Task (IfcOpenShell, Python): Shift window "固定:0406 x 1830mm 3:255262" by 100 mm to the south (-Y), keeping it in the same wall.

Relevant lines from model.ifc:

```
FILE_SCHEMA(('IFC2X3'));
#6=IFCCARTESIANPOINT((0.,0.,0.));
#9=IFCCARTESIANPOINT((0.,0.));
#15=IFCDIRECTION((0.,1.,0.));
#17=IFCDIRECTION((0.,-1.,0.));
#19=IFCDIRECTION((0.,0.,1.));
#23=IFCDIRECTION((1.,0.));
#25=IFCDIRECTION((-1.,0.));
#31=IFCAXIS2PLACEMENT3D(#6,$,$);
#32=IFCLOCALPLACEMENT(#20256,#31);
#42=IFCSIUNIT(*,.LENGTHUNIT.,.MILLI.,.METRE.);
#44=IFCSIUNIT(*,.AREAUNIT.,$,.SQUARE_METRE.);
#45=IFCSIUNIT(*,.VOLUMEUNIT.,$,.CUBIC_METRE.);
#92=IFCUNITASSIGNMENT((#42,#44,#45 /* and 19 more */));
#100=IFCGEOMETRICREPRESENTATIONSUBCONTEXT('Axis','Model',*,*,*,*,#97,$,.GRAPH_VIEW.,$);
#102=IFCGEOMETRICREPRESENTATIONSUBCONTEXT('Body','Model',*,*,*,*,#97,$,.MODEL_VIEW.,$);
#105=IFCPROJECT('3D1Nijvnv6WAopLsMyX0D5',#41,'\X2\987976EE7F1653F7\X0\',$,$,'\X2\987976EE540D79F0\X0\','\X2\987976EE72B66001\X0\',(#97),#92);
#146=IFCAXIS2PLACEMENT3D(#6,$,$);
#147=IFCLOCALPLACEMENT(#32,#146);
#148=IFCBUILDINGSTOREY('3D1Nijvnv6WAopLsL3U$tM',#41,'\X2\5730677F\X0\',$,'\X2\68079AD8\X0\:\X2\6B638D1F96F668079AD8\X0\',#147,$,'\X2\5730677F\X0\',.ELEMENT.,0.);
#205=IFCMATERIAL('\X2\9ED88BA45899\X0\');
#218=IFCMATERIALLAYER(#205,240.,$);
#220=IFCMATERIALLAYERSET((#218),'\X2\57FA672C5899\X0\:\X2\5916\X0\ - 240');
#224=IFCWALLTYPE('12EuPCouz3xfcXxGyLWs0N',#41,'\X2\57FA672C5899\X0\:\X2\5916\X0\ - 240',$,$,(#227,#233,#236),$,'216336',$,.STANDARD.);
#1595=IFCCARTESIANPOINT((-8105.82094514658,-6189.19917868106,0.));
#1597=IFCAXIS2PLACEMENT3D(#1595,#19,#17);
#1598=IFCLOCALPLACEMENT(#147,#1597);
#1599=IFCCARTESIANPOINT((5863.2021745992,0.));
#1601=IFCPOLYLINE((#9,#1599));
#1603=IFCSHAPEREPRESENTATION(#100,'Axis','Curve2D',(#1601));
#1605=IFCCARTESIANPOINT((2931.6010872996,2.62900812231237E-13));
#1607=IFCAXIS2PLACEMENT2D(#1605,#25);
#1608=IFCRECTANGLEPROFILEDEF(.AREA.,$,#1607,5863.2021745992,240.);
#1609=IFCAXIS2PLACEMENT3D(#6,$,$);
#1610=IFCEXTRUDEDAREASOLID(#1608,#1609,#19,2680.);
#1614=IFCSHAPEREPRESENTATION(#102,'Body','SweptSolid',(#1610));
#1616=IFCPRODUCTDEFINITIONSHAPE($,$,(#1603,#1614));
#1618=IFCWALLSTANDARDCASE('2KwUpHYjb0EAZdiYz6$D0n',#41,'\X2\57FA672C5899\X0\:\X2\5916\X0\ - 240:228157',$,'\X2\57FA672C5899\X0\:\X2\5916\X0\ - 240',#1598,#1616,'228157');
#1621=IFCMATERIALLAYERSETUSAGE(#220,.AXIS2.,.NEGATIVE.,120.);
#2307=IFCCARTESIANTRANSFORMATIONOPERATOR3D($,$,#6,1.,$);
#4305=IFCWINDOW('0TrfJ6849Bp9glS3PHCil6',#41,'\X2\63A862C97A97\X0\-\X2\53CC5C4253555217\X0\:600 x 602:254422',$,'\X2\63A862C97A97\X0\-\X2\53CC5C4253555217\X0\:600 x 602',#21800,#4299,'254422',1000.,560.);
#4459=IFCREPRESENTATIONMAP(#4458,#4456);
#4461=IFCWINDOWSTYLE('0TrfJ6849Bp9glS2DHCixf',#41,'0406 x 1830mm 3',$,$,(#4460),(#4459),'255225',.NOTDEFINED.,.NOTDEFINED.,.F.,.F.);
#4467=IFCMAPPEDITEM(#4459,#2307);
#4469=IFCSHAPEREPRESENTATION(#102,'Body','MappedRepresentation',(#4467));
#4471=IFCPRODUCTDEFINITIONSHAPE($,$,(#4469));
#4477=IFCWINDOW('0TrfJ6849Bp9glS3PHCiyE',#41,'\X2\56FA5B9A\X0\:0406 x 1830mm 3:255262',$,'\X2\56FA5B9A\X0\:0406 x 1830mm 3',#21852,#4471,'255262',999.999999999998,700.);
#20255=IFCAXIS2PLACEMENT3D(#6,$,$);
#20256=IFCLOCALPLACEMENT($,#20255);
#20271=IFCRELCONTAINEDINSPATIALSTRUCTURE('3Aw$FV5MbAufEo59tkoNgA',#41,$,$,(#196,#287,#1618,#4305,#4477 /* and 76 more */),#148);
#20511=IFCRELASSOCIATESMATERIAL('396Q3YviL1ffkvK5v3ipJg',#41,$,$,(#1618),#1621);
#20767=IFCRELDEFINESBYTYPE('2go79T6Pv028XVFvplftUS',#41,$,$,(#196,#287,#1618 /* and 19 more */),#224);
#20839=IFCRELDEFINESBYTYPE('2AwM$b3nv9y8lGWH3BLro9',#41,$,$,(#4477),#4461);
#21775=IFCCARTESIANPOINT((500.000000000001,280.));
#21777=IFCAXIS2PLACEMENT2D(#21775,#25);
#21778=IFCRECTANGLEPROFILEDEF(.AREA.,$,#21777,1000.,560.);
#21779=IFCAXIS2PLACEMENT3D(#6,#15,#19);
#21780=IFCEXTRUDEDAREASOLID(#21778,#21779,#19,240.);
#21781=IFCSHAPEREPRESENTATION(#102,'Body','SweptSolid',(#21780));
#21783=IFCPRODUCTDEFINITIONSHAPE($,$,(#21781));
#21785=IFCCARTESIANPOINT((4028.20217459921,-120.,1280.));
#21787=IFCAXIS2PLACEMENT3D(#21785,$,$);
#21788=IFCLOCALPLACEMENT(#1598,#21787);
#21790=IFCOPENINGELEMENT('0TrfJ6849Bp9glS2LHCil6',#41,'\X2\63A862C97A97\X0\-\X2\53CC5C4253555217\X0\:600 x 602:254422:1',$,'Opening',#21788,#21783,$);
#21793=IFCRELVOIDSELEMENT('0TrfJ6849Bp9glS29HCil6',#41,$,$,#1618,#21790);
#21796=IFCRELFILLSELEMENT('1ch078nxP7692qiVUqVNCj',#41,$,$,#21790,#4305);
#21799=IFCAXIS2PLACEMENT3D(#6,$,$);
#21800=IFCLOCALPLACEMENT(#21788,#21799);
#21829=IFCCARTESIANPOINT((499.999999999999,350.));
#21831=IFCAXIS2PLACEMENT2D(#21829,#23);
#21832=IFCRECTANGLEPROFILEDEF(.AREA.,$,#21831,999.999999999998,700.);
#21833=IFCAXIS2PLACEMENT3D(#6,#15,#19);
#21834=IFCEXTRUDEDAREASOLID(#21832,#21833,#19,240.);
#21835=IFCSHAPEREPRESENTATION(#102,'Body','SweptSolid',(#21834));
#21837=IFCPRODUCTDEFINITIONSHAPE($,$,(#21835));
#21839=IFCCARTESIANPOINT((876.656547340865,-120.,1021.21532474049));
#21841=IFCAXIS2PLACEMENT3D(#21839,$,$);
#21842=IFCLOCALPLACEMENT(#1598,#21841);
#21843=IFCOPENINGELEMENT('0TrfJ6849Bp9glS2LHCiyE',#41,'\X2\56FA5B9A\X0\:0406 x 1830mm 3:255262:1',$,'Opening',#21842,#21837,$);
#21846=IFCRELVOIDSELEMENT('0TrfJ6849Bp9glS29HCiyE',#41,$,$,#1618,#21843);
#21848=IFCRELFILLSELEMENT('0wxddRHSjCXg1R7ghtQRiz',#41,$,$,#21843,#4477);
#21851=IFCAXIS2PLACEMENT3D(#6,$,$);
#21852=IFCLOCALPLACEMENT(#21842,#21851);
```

```python
import ifcopenshell
import ifcopenshell.api.geometry
import ifcopenshell.util.placement
import ifcopenshell.util.unit

model = ifcopenshell.open("model.ifc")
unit_scale = ifcopenshell.util.unit.calculate_unit_scale(model)

window = model.by_guid("0TrfJ6849Bp9glS3PHCiyE")
opening = window.FillsVoids[0].RelatingOpeningElement
wall = opening.VoidsElements[0].RelatingBuildingElement

wall_matrix = ifcopenshell.util.placement.get_local_placement(wall.ObjectPlacement)
shift = wall_matrix[:3, 0] * 0.1 / unit_scale
before = ifcopenshell.util.placement.get_local_placement(window.ObjectPlacement)[:3, 3].copy()

# The window is placed relative to its opening, so it follows when the opening moves.
matrix = ifcopenshell.util.placement.get_local_placement(opening.ObjectPlacement)
matrix[:3, 3] += shift
ifcopenshell.api.geometry.edit_object_placement(
    model, product=opening, matrix=matrix, is_si=False, should_transform_children=True
)

after = ifcopenshell.util.placement.get_local_placement(window.ObjectPlacement)[:3, 3]
print("window moved by", (after - before).round(3) + 0.0)

model.write("model_v2.ifc")
```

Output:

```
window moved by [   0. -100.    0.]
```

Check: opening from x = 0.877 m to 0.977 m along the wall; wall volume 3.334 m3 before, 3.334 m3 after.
